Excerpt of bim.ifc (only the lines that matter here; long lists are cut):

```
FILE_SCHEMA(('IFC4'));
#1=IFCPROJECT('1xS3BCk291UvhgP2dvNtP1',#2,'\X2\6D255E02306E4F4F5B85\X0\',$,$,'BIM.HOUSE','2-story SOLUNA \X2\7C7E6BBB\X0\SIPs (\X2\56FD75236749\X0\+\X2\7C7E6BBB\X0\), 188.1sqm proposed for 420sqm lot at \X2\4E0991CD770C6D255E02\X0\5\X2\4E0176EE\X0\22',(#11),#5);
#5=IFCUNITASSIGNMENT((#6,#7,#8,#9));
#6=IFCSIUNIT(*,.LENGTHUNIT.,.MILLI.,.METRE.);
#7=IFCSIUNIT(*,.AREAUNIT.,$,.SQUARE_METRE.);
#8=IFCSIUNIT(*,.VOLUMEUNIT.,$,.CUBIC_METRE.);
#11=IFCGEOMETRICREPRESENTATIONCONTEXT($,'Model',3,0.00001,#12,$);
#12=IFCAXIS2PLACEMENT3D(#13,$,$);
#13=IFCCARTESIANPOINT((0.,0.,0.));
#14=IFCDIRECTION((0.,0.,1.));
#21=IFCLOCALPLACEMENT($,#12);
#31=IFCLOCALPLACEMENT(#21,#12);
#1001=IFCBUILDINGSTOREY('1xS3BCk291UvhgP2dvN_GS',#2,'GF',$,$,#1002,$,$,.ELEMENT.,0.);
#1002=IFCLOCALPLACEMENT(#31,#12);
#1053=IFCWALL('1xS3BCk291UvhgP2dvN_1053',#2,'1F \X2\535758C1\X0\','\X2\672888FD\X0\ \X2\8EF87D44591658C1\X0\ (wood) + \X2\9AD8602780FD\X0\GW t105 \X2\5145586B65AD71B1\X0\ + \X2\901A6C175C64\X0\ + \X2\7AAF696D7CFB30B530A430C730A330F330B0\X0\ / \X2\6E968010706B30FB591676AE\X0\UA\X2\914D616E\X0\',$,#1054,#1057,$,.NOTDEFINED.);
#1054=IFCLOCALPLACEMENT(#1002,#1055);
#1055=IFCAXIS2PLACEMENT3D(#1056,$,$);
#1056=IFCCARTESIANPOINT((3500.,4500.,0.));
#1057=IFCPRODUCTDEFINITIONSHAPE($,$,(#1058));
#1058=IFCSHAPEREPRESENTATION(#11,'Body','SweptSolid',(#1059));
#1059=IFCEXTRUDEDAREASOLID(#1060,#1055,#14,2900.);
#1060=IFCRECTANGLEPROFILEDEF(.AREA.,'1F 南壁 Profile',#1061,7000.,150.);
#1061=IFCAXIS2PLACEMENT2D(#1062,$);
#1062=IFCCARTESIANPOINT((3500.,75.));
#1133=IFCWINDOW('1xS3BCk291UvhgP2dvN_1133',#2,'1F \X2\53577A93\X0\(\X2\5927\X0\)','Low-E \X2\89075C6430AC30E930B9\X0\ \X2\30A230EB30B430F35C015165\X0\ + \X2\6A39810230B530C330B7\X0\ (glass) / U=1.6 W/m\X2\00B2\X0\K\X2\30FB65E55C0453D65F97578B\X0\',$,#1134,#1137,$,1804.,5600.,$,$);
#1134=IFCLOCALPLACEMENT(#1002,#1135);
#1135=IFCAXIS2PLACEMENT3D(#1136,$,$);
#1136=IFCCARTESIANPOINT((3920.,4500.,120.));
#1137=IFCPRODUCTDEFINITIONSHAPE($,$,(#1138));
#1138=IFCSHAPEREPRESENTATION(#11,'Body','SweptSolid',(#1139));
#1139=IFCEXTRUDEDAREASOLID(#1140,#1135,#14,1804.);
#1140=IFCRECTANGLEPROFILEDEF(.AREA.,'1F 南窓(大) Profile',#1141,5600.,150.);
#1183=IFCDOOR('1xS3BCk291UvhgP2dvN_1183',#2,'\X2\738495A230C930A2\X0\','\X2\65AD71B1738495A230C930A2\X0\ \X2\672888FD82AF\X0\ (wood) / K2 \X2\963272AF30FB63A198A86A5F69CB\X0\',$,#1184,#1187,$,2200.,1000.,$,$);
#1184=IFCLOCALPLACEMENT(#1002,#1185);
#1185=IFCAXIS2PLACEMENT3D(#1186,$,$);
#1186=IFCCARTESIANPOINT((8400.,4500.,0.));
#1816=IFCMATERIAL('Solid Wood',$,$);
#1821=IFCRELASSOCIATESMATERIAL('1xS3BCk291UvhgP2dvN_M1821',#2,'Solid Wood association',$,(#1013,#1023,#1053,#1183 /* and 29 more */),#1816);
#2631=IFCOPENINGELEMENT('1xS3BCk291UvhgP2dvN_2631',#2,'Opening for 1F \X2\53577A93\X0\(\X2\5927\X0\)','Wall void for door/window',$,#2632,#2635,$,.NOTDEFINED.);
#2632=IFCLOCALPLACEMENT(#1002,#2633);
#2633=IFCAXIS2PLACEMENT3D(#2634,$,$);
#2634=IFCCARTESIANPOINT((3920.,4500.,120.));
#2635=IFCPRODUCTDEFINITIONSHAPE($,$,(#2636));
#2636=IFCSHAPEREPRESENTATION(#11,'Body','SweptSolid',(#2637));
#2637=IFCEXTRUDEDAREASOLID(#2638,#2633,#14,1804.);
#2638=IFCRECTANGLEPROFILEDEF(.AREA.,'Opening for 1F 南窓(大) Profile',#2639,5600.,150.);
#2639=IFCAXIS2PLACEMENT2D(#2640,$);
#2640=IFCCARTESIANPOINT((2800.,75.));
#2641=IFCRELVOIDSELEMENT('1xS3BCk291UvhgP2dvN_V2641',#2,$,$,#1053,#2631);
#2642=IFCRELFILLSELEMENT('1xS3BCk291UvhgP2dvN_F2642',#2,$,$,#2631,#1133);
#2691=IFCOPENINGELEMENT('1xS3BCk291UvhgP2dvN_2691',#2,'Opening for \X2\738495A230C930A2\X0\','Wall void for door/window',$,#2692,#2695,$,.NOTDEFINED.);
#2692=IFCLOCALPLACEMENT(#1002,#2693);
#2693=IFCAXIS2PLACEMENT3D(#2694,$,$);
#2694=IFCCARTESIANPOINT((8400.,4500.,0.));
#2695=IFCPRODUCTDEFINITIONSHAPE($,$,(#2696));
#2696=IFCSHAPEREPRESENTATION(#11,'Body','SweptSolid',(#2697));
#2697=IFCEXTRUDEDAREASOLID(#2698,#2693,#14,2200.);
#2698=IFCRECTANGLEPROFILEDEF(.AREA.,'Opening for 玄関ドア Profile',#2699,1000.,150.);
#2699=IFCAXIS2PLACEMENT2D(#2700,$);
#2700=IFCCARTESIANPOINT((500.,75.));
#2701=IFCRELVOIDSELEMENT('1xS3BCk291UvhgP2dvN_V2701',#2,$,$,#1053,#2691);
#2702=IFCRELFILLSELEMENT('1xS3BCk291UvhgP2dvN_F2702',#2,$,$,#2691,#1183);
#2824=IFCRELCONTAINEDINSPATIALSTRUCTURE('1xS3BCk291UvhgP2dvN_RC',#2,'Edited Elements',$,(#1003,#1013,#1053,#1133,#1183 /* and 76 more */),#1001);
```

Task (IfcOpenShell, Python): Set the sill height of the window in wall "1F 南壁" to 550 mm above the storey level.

```python
import numpy as np
import ifcopenshell
import ifcopenshell.api.geometry
import ifcopenshell.geom
import ifcopenshell.util.element
import ifcopenshell.util.placement
import ifcopenshell.util.shape
import ifcopenshell.util.unit

model = ifcopenshell.open("bim.ifc")
unit_scale = ifcopenshell.util.unit.calculate_unit_scale(model)

window = model.by_id(1133)
opening = window.FillsVoids[0].RelatingOpeningElement
storey = ifcopenshell.util.element.get_container(window, ifc_class="IfcBuildingStorey")
level = ifcopenshell.util.placement.get_local_placement(storey.ObjectPlacement)[2, 3]

# The opening's origin need not be at the sill, so measure its lowest point.
shape = ifcopenshell.geom.create_shape(ifcopenshell.geom.settings(), opening)
bottom = ifcopenshell.util.shape.get_shape_bottom_elevation(shape, shape.geometry) / unit_scale
dz = level + 550.0 - bottom

shift = np.array([0.0, 0.0, dz])
# The window is not placed relative to its opening, so move both.
for product in (opening, window):
    matrix = ifcopenshell.util.placement.get_local_placement(product.ObjectPlacement)
    matrix[:3, 3] += shift
    ifcopenshell.api.geometry.edit_object_placement(model, product=product, matrix=matrix, is_si=False)

print(f"moved by {dz * unit_scale:+.3f} m")

model.write("bim_updated.ifc")
```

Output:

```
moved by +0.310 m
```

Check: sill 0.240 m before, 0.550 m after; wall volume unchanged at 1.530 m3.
